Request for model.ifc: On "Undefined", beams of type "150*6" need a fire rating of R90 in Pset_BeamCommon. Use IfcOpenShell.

First a look at what the model holds.

```python
import ifcopenshell
import ifcopenshell.util.element

model = ifcopenshell.open("model.ifc")
print(model.schema)
storey = next(s for s in model.by_type("IfcBuildingStorey") if s.Name == "Undefined")
beams = [e for e in ifcopenshell.util.element.get_decomposition(storey) if e.is_a("IfcBeam")]
seen = {}
for e in beams:
    element_type = ifcopenshell.util.element.get_type(e)
    key = (element_type.Name if element_type != e and element_type else None, ifcopenshell.util.element.get_pset(e, "Pset_BeamCommon", "FireRating"))
    seen[key] = seen.get(key, 0) + 1
for (name, value), count in sorted(seen.items(), key=str):
    print(count, "x", name, "|", value)
```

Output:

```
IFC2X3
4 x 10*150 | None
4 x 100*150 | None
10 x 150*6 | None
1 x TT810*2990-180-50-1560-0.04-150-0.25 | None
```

```python
import ifcopenshell
import ifcopenshell.api.pset
import ifcopenshell.util.element

model = ifcopenshell.open("model.ifc")

storey = next(s for s in model.by_type("IfcBuildingStorey") if s.Name == "Undefined")
beams = [e for e in ifcopenshell.util.element.get_decomposition(storey) if e.is_a("IfcBeam")]

count = 0
for e in beams:
    element_type = ifcopenshell.util.element.get_type(e)
    if element_type in (None, e) or element_type.Name != "150*6":
        continue
    # add_pset returns the element's existing set when there is one.
    pset = ifcopenshell.api.pset.add_pset(model, product=e, name="Pset_BeamCommon")
    ifcopenshell.api.pset.edit_pset(model, pset=pset, properties={"FireRating": "R90"})
    count += 1

print(count, "beams updated")

model.write("model_edited.ifc")
```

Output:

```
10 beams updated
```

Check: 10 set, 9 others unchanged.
